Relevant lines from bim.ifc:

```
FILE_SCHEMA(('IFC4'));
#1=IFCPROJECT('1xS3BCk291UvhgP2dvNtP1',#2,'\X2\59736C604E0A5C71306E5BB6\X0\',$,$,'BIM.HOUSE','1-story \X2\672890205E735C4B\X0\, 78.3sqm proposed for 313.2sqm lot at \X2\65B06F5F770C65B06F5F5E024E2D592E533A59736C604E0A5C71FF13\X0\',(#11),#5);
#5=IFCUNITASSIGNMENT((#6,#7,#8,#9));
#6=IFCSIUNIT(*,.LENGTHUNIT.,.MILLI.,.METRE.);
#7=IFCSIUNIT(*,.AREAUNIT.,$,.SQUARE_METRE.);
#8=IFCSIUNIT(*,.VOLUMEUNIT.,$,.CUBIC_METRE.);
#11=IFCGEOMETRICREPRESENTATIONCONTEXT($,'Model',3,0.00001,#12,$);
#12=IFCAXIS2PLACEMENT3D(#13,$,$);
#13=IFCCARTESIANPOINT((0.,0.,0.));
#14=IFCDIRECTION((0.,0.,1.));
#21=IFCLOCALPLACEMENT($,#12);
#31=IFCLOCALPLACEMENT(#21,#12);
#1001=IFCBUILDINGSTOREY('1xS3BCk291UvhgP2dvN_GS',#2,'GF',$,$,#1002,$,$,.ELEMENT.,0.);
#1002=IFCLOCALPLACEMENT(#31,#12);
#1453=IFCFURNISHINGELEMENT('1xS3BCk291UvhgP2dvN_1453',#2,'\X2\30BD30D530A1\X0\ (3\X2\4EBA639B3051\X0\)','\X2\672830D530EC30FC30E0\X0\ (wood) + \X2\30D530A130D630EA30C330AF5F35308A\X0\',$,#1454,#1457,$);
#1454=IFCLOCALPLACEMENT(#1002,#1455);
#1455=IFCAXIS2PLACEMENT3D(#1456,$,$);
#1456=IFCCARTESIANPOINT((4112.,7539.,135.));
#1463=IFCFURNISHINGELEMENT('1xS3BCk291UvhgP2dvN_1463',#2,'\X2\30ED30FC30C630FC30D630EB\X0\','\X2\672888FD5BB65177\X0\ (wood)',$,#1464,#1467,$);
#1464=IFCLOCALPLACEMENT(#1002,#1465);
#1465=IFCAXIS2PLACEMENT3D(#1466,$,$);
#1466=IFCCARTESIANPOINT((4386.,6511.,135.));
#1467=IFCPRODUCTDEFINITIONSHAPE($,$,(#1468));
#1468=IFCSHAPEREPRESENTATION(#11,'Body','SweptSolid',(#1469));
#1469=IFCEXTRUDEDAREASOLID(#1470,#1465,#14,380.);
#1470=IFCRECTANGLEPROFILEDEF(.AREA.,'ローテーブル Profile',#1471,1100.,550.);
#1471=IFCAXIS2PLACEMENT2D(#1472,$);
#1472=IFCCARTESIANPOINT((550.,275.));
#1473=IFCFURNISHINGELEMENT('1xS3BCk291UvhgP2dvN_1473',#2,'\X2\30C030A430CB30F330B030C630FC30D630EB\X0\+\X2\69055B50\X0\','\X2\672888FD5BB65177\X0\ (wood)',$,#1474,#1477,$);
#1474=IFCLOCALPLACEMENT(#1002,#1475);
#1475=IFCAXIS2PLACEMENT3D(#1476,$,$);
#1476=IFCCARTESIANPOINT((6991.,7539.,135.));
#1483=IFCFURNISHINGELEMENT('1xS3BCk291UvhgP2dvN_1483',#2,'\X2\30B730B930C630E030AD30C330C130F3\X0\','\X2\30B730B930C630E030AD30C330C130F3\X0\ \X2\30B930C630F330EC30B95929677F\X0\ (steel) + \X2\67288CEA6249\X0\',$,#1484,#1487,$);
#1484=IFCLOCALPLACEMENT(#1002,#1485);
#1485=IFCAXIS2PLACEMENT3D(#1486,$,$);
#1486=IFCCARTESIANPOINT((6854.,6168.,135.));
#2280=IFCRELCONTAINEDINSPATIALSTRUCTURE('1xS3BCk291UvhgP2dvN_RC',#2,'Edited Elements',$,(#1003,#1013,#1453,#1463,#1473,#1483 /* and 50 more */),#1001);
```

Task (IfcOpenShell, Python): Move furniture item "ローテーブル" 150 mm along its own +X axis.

```python
import ifcopenshell
import ifcopenshell.api.geometry
import ifcopenshell.util.placement
import ifcopenshell.util.unit

model = ifcopenshell.open("bim.ifc")
unit_scale = ifcopenshell.util.unit.calculate_unit_scale(model)

item = model.by_guid("1xS3BCk291UvhgP2dvN_1463")
matrix = ifcopenshell.util.placement.get_local_placement(item.ObjectPlacement)
matrix[:3, 3] += matrix[:3, 0] * 0.15 / unit_scale
ifcopenshell.api.geometry.edit_object_placement(model, product=item, matrix=matrix, is_si=False)

print(ifcopenshell.util.placement.get_local_placement(item.ObjectPlacement).round(3) + 0.0)

model.write("bim-out.ifc")
```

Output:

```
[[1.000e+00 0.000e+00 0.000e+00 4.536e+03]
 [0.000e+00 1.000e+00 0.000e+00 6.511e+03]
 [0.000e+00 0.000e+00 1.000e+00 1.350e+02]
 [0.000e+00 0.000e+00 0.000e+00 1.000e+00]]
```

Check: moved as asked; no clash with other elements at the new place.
